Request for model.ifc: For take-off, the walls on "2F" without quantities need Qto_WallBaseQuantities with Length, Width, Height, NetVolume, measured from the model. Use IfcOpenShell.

First a look at what the model holds.

```python
import ifcopenshell
import ifcopenshell.util.element
import ifcopenshell.util.unit

model = ifcopenshell.open("model.ifc")
print(model.schema)
for unit_type in ("LENGTHUNIT", "AREAUNIT", "VOLUMEUNIT"):
    print(unit_type, ifcopenshell.util.unit.calculate_unit_scale(model, unit_type))
storey = next(s for s in model.by_type("IfcBuildingStorey") if s.Name == "2F")
walls = [e for e in ifcopenshell.util.element.get_decomposition(storey) if e.is_a("IfcWall")]
for e in sorted(walls, key=lambda e: e.id()):
    print(e.id(), e.is_a(), e.Name, list(ifcopenshell.util.element.get_psets(e, qtos_only=True)), sep=" | ")
```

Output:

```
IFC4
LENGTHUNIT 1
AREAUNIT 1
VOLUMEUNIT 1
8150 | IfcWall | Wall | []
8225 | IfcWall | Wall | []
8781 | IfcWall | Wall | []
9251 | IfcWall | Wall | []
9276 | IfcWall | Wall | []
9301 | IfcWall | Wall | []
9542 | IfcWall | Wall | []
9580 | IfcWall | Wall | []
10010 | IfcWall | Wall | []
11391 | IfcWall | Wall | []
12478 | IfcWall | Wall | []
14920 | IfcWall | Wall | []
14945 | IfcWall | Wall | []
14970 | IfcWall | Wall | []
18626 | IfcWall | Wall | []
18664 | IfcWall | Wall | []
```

```python
import ifcopenshell
import ifcopenshell.api.pset
import ifcopenshell.geom
import ifcopenshell.util.element
import ifcopenshell.util.shape
import ifcopenshell.util.unit

model = ifcopenshell.open("model.ifc")
unit_scale = ifcopenshell.util.unit.calculate_unit_scale(model)
volume_scale = ifcopenshell.util.unit.calculate_unit_scale(model, "VOLUMEUNIT")
settings = ifcopenshell.geom.settings()

storey = next(s for s in model.by_type("IfcBuildingStorey") if s.Name == "2F")
walls = [e for e in ifcopenshell.util.element.get_decomposition(storey) if e.is_a("IfcWall")]

for e in sorted(walls, key=lambda e: e.id()):
    if ifcopenshell.util.element.get_psets(e, qtos_only=True, should_inherit=False):
        continue
    # Geometry comes back in metres, in the element's own axes.
    shape = ifcopenshell.geom.create_shape(settings, e)
    values = {
        "Length": ifcopenshell.util.shape.get_x(shape.geometry) / unit_scale,
        "Width": ifcopenshell.util.shape.get_y(shape.geometry) / unit_scale,
        "Height": ifcopenshell.util.shape.get_z(shape.geometry) / unit_scale,
        "NetVolume": ifcopenshell.util.shape.get_volume(shape.geometry) / volume_scale,
    }
    qto = ifcopenshell.api.pset.add_qto(model, product=e, name="Qto_WallBaseQuantities")
    ifcopenshell.api.pset.edit_qto(model, qto=qto, properties=values)
    print(e.id(), {k: round(v, 3) for k, v in values.items()})

model.write("model_v2.ifc")
```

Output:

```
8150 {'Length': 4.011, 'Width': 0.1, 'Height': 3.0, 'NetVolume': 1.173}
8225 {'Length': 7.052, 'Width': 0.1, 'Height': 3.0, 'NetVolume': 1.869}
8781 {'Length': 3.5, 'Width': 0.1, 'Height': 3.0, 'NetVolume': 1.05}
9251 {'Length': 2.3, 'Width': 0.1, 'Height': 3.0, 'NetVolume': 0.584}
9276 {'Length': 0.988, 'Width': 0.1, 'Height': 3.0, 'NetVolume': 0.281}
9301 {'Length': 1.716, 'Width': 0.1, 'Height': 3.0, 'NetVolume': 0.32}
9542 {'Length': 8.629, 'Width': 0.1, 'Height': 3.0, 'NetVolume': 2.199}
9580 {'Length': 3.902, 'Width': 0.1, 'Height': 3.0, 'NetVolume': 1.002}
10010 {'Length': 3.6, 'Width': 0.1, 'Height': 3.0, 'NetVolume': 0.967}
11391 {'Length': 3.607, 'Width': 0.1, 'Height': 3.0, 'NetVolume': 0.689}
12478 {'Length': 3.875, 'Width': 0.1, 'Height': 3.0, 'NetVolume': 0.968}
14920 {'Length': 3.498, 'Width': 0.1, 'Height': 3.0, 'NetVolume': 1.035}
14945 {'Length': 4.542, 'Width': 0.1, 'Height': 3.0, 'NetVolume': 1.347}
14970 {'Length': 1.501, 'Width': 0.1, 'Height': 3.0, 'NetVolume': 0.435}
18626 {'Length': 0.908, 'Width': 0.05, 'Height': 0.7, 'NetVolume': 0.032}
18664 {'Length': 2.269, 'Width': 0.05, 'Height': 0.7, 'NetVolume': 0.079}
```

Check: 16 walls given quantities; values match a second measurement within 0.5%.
